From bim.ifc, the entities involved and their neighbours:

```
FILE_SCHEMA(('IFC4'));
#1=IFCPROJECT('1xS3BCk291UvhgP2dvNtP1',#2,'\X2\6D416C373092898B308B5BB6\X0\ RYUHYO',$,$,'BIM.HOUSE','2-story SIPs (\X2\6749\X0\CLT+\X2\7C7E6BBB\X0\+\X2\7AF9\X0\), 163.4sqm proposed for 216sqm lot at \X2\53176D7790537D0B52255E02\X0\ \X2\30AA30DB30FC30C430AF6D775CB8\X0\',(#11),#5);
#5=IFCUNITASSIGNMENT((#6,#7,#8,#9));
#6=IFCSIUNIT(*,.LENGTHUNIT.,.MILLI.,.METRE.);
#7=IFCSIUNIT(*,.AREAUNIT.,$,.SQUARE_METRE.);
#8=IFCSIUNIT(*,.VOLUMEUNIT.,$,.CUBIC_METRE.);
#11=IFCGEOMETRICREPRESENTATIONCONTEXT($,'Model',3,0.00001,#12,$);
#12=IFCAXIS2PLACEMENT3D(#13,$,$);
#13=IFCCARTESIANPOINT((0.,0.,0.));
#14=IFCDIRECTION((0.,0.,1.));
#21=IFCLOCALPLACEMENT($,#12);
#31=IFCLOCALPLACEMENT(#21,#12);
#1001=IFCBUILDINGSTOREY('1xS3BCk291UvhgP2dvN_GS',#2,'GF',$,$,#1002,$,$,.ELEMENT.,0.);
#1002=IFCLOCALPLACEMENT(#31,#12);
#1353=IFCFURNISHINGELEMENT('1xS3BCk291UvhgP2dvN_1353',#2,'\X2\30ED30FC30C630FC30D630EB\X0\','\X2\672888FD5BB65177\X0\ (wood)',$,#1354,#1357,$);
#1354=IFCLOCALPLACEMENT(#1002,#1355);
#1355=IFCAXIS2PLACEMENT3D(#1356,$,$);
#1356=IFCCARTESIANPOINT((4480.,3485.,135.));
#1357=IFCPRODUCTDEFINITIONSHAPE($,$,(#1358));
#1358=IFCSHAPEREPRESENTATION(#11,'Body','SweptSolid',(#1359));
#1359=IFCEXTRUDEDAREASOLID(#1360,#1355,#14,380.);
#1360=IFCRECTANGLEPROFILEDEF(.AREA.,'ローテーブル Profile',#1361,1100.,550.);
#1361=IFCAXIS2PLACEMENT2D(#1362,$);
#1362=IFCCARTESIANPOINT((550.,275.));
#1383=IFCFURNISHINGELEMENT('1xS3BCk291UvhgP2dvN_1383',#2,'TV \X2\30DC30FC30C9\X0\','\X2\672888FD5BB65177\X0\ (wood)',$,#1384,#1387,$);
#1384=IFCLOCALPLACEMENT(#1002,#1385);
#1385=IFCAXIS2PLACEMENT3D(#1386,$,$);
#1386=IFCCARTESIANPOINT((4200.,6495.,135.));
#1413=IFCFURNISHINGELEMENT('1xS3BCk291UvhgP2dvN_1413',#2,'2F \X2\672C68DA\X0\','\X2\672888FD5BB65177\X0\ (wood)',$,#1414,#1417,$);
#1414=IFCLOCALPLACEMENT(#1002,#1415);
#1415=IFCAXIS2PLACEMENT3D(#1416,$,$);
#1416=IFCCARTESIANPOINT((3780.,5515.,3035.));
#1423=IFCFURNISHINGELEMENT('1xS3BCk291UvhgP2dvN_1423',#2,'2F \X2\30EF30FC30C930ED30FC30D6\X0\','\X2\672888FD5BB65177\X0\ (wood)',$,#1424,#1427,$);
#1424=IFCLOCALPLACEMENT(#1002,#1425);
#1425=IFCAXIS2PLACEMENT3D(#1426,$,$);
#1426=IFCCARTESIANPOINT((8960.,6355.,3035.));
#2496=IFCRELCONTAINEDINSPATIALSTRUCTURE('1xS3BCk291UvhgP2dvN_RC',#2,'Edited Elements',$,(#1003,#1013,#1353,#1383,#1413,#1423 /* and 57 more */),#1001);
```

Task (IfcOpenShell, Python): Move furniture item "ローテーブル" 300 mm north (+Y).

```python
import ifcopenshell
import ifcopenshell.api.geometry
import ifcopenshell.util.placement
import ifcopenshell.util.unit

model = ifcopenshell.open("bim.ifc")
unit_scale = ifcopenshell.util.unit.calculate_unit_scale(model)

item = model.by_guid("1xS3BCk291UvhgP2dvN_1353")
matrix = ifcopenshell.util.placement.get_local_placement(item.ObjectPlacement)
matrix[1, 3] += 0.3 / unit_scale
ifcopenshell.api.geometry.edit_object_placement(model, product=item, matrix=matrix, is_si=False)

print(ifcopenshell.util.placement.get_local_placement(item.ObjectPlacement).round(3) + 0.0)

model.write("bim-out.ifc")
```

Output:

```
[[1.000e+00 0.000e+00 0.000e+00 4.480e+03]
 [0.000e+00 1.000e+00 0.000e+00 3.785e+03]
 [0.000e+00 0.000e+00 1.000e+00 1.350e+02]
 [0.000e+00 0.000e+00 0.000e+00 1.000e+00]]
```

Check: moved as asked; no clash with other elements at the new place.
